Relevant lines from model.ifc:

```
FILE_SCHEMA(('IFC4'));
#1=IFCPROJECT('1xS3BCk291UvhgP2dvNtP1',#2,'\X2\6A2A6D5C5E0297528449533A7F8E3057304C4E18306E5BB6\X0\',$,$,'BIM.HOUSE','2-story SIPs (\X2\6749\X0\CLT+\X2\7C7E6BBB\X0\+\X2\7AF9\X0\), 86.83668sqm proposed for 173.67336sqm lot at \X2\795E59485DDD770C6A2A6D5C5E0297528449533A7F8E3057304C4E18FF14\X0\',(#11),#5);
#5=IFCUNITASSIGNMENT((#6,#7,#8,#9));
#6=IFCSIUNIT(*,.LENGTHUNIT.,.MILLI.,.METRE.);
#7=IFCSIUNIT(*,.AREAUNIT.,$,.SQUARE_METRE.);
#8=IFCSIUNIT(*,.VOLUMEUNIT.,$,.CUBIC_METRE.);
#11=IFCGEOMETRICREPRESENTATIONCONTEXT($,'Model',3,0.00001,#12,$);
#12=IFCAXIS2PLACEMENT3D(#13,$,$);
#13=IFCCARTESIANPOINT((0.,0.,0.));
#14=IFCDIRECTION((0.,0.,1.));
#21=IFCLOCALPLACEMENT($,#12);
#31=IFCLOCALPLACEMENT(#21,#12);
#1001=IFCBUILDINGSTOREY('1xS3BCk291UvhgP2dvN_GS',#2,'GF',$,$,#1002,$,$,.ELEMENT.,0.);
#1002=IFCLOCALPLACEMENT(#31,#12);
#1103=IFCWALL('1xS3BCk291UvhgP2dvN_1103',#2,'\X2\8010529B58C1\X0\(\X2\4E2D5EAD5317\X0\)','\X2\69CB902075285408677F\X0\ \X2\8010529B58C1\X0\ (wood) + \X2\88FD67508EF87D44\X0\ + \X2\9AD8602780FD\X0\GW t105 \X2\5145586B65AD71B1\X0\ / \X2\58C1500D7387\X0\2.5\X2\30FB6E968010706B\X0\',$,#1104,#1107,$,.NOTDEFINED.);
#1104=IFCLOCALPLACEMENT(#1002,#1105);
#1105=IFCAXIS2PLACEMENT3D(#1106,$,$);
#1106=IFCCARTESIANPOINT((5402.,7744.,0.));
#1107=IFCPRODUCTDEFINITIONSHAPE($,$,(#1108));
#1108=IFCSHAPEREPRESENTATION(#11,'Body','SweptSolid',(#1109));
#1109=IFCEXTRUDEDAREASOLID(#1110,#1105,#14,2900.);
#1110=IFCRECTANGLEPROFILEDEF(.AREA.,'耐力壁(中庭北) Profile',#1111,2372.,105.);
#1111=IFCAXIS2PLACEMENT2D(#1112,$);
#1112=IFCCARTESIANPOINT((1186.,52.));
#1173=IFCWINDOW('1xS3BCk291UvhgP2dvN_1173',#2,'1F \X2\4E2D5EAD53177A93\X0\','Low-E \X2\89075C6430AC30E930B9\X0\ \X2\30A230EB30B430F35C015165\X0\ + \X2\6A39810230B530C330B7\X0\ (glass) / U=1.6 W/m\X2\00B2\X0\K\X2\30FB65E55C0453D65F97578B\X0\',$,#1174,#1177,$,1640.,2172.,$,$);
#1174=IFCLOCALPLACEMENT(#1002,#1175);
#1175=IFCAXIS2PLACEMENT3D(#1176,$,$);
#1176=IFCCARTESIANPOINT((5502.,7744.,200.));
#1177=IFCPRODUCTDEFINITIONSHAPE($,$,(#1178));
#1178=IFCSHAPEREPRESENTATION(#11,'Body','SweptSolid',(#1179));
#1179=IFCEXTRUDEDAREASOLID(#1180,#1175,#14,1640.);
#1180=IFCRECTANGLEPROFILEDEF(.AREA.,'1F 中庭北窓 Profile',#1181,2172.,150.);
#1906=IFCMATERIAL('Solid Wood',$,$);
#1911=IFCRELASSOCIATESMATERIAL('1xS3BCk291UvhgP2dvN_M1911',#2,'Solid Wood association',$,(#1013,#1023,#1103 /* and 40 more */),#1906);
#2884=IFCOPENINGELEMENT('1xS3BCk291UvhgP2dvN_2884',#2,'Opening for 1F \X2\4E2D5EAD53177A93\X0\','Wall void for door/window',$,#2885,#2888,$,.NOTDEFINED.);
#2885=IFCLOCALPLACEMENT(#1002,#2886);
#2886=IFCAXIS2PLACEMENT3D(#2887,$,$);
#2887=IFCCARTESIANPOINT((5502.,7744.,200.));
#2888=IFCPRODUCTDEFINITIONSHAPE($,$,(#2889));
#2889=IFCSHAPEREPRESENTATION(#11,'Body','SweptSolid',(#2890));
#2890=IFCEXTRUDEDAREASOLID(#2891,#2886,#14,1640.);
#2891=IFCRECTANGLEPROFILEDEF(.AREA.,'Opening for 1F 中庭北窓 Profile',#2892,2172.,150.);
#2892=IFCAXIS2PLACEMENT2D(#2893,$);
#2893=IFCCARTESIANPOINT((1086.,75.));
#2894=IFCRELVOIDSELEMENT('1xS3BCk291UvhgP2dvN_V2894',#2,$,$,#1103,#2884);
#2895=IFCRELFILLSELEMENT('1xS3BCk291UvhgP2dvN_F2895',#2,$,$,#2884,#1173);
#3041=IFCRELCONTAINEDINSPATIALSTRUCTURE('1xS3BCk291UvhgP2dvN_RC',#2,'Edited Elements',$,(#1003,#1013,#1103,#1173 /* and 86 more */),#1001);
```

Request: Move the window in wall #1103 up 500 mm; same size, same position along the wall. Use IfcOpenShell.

```python
import numpy as np
import ifcopenshell
import ifcopenshell.api.geometry
import ifcopenshell.util.placement
import ifcopenshell.util.unit

model = ifcopenshell.open("model.ifc")
unit_scale = ifcopenshell.util.unit.calculate_unit_scale(model)

window = model.by_guid("1xS3BCk291UvhgP2dvN_1173")
opening = window.FillsVoids[0].RelatingOpeningElement
dz = 0.5 / unit_scale

shift = np.array([0.0, 0.0, dz])
# The window is not placed relative to its opening, so move both.
for product in (opening, window):
    matrix = ifcopenshell.util.placement.get_local_placement(product.ObjectPlacement)
    matrix[:3, 3] += shift
    ifcopenshell.api.geometry.edit_object_placement(model, product=product, matrix=matrix, is_si=False)

print(f"moved by {dz * unit_scale:+.3f} m")

model.write("model-out.ifc")
```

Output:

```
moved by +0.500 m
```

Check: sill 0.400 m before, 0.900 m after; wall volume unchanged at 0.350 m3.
